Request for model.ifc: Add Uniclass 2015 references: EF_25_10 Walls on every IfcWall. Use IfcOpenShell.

First a look at what the model holds.

```python
import ifcopenshell

model = ifcopenshell.open("model.ifc")
print(model.schema)
print("classifications:", [c.Name for c in model.by_type("IfcClassification")])
for ifc_class in ("IfcDoor", "IfcRoof", "IfcStair", "IfcWall", "IfcWindow"):
    print(ifc_class, len(model.by_type(ifc_class)))
```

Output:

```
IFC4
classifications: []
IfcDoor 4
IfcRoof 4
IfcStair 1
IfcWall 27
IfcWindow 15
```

```python
import ifcopenshell
import ifcopenshell.api.classification

model = ifcopenshell.open("model.ifc")

system = ifcopenshell.api.classification.add_classification(model, classification="Uniclass 2015")

codes = {
    "IfcWall": ("EF_25_10", "Walls"),
}
for ifc_class, (code, name) in codes.items():
    products = model.by_type(ifc_class)
    ifcopenshell.api.classification.add_reference(
        model, products=products, classification=system, identification=code, name=name
    )
    print(code, len(products))

model.write("model_v2.ifc")
```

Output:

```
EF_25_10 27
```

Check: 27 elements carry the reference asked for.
